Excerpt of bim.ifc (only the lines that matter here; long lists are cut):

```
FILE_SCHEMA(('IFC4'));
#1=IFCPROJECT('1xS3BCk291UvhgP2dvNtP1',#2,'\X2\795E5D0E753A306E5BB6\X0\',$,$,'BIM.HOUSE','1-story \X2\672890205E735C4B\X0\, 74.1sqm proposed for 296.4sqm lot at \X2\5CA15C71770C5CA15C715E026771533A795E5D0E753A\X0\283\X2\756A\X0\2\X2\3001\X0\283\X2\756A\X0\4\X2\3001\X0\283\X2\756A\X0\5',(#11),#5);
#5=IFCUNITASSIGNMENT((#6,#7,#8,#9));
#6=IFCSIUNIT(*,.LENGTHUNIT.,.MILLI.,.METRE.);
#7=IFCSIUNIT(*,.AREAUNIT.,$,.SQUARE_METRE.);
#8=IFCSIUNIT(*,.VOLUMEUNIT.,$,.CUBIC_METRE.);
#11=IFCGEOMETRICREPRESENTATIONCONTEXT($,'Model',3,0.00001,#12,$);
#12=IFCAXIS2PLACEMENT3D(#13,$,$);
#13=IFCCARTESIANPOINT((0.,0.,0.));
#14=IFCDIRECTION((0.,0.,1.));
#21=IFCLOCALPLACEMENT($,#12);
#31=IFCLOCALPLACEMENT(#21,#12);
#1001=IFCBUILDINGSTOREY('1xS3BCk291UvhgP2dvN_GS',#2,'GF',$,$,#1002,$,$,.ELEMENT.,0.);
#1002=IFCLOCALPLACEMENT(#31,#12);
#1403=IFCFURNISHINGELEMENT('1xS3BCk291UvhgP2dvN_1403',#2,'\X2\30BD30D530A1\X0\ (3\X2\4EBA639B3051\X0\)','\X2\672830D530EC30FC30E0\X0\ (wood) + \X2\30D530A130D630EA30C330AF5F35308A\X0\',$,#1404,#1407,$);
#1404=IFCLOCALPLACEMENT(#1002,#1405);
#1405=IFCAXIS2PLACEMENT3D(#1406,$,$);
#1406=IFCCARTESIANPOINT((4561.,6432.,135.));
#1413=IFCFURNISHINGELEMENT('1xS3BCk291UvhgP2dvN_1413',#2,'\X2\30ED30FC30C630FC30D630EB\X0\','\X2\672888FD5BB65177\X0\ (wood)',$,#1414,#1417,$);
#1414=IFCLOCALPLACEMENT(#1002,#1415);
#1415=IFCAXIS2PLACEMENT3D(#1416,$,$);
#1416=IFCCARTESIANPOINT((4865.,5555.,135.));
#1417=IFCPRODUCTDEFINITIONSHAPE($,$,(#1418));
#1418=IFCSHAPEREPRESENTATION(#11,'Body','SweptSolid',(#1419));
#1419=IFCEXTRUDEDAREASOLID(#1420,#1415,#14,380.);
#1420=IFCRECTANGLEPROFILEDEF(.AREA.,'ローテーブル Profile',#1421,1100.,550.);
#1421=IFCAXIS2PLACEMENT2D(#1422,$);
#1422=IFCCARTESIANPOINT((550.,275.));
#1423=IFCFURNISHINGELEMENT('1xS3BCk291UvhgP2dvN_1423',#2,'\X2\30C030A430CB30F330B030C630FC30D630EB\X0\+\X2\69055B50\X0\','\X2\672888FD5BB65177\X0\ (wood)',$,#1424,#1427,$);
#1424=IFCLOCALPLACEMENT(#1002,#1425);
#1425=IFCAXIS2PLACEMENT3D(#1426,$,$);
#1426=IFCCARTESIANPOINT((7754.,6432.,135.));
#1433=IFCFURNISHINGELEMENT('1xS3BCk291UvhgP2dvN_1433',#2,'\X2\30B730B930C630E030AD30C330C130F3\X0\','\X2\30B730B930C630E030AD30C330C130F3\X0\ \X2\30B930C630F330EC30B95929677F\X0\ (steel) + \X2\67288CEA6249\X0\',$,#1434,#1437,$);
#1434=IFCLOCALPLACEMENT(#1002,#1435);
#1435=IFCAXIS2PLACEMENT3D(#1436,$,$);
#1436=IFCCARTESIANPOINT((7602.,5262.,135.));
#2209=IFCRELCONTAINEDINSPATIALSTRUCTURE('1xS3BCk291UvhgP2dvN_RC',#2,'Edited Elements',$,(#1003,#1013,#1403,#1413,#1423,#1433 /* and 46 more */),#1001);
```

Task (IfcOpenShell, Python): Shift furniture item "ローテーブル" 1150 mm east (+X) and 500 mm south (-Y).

```python
import ifcopenshell
import ifcopenshell.api.geometry
import ifcopenshell.util.placement
import ifcopenshell.util.unit

model = ifcopenshell.open("bim.ifc")
unit_scale = ifcopenshell.util.unit.calculate_unit_scale(model)

item = model.by_id(1413)
matrix = ifcopenshell.util.placement.get_local_placement(item.ObjectPlacement)
matrix[0, 3] += 1.15 / unit_scale
matrix[1, 3] -= 0.5 / unit_scale
ifcopenshell.api.geometry.edit_object_placement(model, product=item, matrix=matrix, is_si=False)

print(ifcopenshell.util.placement.get_local_placement(item.ObjectPlacement).round(3) + 0.0)

model.write("bim_updated.ifc")
```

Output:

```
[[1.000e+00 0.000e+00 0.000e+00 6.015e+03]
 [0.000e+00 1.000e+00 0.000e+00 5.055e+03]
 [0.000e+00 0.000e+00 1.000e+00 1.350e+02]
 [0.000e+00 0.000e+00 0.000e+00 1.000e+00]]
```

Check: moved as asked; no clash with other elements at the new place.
